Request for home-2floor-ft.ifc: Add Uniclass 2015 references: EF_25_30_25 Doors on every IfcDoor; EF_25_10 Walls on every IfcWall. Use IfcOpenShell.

First a look at what the model holds.

```python
import ifcopenshell

model = ifcopenshell.open("home-2floor-ft.ifc")
print(model.schema)
print("classifications:", [c.Name for c in model.by_type("IfcClassification")])
for ifc_class in ("IfcDoor", "IfcRoof", "IfcStair", "IfcWall", "IfcWindow"):
    print(ifc_class, len(model.by_type(ifc_class)))
```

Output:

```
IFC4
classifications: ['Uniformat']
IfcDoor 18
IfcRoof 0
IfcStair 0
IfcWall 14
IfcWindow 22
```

```python
import ifcopenshell
import ifcopenshell.api.classification

model = ifcopenshell.open("home-2floor-ft.ifc")

system = ifcopenshell.api.classification.add_classification(model, classification="Uniclass 2015")

codes = {
    "IfcDoor": ("EF_25_30_25", "Doors"),
    "IfcWall": ("EF_25_10", "Walls"),
}
for ifc_class, (code, name) in codes.items():
    products = model.by_type(ifc_class)
    ifcopenshell.api.classification.add_reference(
        model, products=products, classification=system, identification=code, name=name
    )
    print(code, len(products))

model.write("home-2floor-ft_rev.ifc")
```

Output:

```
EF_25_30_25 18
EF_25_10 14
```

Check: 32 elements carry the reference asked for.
